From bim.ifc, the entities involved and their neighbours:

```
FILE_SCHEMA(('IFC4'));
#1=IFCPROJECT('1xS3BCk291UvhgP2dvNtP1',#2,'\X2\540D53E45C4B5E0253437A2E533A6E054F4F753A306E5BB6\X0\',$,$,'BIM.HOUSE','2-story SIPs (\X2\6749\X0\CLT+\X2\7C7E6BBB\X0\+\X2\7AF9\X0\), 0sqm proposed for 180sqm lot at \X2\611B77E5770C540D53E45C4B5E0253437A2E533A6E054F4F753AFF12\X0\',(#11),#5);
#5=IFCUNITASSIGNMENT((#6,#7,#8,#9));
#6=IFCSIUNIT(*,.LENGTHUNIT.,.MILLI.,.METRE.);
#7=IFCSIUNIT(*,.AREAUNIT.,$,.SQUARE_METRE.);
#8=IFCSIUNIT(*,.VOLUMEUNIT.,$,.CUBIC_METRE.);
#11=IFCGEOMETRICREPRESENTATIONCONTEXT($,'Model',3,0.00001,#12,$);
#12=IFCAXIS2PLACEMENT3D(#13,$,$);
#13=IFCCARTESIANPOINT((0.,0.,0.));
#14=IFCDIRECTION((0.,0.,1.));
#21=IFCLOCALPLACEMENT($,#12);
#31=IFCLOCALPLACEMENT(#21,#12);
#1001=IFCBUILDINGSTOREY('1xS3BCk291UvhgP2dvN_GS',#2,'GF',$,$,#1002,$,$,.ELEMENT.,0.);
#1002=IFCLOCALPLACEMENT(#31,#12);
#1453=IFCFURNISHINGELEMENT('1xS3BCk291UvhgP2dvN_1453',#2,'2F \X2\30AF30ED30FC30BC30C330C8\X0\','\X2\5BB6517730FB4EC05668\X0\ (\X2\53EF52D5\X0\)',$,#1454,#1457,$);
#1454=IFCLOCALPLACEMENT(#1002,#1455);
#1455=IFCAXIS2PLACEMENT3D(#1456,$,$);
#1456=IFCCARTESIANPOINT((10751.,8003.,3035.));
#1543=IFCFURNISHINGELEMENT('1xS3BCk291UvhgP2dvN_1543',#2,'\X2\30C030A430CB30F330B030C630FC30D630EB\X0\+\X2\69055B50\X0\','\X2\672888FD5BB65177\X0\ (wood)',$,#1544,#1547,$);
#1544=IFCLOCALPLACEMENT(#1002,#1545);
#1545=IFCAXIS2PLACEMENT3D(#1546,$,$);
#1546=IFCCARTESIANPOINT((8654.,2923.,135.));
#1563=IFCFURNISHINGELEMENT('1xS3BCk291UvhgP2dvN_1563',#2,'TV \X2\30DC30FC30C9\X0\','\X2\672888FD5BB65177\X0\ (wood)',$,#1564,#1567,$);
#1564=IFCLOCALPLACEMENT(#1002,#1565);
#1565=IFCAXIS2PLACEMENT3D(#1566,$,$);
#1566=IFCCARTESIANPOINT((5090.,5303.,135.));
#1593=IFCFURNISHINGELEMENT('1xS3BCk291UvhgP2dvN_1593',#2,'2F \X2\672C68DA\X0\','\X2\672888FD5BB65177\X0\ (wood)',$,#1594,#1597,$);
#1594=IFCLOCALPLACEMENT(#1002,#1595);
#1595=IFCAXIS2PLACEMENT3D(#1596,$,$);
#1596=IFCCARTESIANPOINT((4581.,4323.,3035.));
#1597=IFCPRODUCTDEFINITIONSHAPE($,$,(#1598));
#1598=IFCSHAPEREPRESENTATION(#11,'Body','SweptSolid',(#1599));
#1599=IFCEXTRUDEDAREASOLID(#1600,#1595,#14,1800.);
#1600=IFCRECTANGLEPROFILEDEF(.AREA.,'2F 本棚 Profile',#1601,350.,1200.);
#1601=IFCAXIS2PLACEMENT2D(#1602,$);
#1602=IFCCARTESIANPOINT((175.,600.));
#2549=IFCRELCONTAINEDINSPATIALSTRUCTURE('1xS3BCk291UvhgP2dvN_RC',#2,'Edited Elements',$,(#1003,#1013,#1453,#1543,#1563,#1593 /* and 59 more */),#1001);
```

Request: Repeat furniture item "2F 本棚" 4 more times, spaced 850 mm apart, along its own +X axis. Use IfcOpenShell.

```python
import ifcopenshell
import ifcopenshell.api.geometry
import ifcopenshell.api.root
import ifcopenshell.util.element
import ifcopenshell.util.placement
import ifcopenshell.util.unit

model = ifcopenshell.open("bim.ifc")
unit_scale = ifcopenshell.util.unit.calculate_unit_scale(model)


def reuse_history(source, copy):
    """copy_class also copies each property set's owner history, people and application; keep the originals."""
    for rel in copy.IsDefinedBy:
        if rel.is_a("IfcRelDefinesByProperties") and (history := rel.RelatingPropertyDefinition.OwnerHistory):
            rel.RelatingPropertyDefinition.OwnerHistory = source.OwnerHistory
            ifcopenshell.util.element.remove_deep2(model, history)


source = model.by_guid("1xS3BCk291UvhgP2dvN_1593")
base = ifcopenshell.util.placement.get_local_placement(source.ObjectPlacement)
step = base[:3, 0] * 0.85 / unit_scale

for i in range(1, 5):
    copy = ifcopenshell.api.root.copy_class(model, product=source)
    copy.Representation = ifcopenshell.util.element.copy_deep(
        model, source.Representation, exclude=["IfcGeometricRepresentationContext", "IfcRepresentationMap"]
    )
    reuse_history(source, copy)
    matrix = base.copy()
    matrix[:3, 3] += i * step
    print("added at", matrix[:3, 3].round(3) + 0.0)
    ifcopenshell.api.geometry.edit_object_placement(model, product=copy, matrix=matrix, is_si=False)

model.write("bim_updated.ifc")
```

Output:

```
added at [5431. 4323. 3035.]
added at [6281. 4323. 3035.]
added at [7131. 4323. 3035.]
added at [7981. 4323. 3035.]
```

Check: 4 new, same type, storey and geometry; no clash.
